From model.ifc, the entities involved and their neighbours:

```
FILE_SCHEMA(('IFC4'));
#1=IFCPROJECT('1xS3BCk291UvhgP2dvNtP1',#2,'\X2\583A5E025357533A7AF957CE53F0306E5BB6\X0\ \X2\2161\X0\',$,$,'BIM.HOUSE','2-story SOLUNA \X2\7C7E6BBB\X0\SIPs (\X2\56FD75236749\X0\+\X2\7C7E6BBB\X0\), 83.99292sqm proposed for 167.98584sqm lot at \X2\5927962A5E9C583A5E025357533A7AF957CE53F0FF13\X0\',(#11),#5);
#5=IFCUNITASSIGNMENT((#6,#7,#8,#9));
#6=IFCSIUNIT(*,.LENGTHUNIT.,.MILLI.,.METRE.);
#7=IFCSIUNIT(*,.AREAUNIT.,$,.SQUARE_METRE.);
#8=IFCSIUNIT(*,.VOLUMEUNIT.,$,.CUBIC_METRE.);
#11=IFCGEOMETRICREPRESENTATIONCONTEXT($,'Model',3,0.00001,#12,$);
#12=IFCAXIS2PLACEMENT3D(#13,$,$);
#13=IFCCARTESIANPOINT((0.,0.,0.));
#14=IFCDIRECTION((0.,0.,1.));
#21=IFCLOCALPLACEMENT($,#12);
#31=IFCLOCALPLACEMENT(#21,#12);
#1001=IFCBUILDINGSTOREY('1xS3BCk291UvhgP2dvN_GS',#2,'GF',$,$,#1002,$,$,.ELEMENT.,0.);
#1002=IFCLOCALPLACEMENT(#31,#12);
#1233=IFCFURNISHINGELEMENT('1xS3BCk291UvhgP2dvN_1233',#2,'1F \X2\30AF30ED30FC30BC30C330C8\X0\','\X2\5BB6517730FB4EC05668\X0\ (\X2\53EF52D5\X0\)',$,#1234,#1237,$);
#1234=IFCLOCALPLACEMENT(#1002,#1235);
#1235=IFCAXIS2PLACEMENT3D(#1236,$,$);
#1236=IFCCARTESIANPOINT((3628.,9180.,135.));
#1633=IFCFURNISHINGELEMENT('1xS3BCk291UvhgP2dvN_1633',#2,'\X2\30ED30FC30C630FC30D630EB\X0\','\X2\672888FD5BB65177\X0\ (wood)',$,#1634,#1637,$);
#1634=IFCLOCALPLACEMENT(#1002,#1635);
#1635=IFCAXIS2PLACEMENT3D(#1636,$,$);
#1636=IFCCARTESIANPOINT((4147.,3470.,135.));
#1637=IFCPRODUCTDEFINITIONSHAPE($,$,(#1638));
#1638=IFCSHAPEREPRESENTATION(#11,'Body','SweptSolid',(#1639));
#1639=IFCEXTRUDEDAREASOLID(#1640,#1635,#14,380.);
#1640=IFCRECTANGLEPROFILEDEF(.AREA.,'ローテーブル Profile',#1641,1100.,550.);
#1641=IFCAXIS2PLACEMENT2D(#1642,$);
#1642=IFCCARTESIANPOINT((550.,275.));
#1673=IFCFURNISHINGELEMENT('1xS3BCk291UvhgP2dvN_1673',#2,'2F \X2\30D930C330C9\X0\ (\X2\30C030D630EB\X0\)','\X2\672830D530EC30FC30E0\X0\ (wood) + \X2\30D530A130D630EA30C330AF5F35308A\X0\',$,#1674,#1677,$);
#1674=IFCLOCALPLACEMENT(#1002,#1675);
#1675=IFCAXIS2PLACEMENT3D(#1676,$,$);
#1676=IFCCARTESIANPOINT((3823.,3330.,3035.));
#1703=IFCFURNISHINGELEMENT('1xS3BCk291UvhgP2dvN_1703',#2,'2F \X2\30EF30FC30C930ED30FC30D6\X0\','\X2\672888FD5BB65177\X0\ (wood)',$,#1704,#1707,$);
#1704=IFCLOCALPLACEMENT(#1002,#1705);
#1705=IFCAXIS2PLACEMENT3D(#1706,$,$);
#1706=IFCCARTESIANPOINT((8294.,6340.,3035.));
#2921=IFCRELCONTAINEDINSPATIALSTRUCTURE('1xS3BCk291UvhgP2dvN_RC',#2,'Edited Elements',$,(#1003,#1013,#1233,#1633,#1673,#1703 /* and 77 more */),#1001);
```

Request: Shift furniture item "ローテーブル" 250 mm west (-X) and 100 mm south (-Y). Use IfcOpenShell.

```python
import ifcopenshell
import ifcopenshell.api.geometry
import ifcopenshell.util.placement

model = ifcopenshell.open("model.ifc")

item = model.by_guid("1xS3BCk291UvhgP2dvN_1633")
matrix = ifcopenshell.util.placement.get_local_placement(item.ObjectPlacement)
matrix[0, 3] -= 250.0
matrix[1, 3] -= 100.0
ifcopenshell.api.geometry.edit_object_placement(model, product=item, matrix=matrix, is_si=False)

print(ifcopenshell.util.placement.get_local_placement(item.ObjectPlacement).round(3) + 0.0)

model.write("model-out.ifc")
```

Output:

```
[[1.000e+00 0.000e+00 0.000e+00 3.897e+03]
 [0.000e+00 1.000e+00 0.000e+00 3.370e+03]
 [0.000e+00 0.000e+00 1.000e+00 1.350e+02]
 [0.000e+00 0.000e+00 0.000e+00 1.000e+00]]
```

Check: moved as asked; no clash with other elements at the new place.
